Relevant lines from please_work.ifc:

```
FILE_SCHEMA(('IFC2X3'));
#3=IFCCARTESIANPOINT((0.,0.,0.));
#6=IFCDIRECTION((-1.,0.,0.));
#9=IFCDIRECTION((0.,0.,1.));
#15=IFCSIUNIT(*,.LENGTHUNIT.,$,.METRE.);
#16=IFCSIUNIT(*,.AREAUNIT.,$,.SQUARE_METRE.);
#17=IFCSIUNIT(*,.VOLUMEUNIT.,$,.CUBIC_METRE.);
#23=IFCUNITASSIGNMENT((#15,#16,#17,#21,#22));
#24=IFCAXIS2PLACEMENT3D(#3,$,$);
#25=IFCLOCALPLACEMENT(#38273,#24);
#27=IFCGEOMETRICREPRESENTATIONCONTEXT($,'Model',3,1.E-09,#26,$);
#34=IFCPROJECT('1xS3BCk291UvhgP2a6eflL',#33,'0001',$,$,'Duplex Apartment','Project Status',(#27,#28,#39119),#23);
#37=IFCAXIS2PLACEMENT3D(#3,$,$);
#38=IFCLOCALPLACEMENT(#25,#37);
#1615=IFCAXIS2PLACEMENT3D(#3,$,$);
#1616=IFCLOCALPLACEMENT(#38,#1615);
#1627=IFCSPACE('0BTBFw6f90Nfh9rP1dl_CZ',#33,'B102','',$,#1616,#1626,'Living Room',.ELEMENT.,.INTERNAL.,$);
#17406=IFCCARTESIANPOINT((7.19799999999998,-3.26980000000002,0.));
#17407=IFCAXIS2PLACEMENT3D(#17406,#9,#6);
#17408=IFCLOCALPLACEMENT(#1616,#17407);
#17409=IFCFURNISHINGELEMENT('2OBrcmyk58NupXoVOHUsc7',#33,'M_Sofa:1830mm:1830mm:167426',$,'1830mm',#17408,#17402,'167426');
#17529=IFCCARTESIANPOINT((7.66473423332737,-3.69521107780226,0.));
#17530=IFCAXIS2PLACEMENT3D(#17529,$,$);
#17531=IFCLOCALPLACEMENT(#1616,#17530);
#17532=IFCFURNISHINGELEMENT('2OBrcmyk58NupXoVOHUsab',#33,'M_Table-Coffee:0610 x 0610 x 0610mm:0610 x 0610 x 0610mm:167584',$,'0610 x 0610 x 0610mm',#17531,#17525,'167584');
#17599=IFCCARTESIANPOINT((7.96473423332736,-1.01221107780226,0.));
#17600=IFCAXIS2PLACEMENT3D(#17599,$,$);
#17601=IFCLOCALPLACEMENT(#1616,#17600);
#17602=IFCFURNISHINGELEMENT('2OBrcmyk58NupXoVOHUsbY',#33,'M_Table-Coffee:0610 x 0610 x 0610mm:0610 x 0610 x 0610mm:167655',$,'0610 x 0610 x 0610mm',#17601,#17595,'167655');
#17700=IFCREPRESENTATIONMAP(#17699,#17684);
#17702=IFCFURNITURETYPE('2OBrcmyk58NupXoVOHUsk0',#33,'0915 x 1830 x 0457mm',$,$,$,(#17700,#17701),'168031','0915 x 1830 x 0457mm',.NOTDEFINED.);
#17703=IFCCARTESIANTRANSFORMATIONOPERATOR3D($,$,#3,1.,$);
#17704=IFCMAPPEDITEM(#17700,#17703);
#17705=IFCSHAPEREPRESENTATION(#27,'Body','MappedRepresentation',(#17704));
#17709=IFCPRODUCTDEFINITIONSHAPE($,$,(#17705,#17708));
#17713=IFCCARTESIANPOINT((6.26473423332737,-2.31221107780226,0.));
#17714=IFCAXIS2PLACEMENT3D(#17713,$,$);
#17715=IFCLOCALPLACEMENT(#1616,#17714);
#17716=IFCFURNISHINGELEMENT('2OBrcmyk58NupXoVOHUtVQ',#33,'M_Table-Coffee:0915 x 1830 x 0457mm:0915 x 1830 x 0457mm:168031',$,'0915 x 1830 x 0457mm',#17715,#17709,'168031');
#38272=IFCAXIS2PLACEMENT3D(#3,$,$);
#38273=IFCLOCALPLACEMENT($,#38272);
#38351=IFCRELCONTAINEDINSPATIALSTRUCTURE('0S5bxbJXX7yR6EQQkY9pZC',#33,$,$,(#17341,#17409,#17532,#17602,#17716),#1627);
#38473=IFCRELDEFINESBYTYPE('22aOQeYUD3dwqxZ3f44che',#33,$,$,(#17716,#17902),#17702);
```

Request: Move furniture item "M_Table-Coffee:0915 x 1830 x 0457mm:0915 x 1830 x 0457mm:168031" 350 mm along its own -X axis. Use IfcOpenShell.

```python
import ifcopenshell
import ifcopenshell.api.geometry
import ifcopenshell.util.placement

model = ifcopenshell.open("please_work.ifc")

item = model.by_guid("2OBrcmyk58NupXoVOHUtVQ")
matrix = ifcopenshell.util.placement.get_local_placement(item.ObjectPlacement)
matrix[:3, 3] -= matrix[:3, 0] * 0.35
ifcopenshell.api.geometry.edit_object_placement(model, product=item, matrix=matrix, is_si=False)

print(ifcopenshell.util.placement.get_local_placement(item.ObjectPlacement).round(3) + 0.0)

model.write("please_work_edited.ifc")
```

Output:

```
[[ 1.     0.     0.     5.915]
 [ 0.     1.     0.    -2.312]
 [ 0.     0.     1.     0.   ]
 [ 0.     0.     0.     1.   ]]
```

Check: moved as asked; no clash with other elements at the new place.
